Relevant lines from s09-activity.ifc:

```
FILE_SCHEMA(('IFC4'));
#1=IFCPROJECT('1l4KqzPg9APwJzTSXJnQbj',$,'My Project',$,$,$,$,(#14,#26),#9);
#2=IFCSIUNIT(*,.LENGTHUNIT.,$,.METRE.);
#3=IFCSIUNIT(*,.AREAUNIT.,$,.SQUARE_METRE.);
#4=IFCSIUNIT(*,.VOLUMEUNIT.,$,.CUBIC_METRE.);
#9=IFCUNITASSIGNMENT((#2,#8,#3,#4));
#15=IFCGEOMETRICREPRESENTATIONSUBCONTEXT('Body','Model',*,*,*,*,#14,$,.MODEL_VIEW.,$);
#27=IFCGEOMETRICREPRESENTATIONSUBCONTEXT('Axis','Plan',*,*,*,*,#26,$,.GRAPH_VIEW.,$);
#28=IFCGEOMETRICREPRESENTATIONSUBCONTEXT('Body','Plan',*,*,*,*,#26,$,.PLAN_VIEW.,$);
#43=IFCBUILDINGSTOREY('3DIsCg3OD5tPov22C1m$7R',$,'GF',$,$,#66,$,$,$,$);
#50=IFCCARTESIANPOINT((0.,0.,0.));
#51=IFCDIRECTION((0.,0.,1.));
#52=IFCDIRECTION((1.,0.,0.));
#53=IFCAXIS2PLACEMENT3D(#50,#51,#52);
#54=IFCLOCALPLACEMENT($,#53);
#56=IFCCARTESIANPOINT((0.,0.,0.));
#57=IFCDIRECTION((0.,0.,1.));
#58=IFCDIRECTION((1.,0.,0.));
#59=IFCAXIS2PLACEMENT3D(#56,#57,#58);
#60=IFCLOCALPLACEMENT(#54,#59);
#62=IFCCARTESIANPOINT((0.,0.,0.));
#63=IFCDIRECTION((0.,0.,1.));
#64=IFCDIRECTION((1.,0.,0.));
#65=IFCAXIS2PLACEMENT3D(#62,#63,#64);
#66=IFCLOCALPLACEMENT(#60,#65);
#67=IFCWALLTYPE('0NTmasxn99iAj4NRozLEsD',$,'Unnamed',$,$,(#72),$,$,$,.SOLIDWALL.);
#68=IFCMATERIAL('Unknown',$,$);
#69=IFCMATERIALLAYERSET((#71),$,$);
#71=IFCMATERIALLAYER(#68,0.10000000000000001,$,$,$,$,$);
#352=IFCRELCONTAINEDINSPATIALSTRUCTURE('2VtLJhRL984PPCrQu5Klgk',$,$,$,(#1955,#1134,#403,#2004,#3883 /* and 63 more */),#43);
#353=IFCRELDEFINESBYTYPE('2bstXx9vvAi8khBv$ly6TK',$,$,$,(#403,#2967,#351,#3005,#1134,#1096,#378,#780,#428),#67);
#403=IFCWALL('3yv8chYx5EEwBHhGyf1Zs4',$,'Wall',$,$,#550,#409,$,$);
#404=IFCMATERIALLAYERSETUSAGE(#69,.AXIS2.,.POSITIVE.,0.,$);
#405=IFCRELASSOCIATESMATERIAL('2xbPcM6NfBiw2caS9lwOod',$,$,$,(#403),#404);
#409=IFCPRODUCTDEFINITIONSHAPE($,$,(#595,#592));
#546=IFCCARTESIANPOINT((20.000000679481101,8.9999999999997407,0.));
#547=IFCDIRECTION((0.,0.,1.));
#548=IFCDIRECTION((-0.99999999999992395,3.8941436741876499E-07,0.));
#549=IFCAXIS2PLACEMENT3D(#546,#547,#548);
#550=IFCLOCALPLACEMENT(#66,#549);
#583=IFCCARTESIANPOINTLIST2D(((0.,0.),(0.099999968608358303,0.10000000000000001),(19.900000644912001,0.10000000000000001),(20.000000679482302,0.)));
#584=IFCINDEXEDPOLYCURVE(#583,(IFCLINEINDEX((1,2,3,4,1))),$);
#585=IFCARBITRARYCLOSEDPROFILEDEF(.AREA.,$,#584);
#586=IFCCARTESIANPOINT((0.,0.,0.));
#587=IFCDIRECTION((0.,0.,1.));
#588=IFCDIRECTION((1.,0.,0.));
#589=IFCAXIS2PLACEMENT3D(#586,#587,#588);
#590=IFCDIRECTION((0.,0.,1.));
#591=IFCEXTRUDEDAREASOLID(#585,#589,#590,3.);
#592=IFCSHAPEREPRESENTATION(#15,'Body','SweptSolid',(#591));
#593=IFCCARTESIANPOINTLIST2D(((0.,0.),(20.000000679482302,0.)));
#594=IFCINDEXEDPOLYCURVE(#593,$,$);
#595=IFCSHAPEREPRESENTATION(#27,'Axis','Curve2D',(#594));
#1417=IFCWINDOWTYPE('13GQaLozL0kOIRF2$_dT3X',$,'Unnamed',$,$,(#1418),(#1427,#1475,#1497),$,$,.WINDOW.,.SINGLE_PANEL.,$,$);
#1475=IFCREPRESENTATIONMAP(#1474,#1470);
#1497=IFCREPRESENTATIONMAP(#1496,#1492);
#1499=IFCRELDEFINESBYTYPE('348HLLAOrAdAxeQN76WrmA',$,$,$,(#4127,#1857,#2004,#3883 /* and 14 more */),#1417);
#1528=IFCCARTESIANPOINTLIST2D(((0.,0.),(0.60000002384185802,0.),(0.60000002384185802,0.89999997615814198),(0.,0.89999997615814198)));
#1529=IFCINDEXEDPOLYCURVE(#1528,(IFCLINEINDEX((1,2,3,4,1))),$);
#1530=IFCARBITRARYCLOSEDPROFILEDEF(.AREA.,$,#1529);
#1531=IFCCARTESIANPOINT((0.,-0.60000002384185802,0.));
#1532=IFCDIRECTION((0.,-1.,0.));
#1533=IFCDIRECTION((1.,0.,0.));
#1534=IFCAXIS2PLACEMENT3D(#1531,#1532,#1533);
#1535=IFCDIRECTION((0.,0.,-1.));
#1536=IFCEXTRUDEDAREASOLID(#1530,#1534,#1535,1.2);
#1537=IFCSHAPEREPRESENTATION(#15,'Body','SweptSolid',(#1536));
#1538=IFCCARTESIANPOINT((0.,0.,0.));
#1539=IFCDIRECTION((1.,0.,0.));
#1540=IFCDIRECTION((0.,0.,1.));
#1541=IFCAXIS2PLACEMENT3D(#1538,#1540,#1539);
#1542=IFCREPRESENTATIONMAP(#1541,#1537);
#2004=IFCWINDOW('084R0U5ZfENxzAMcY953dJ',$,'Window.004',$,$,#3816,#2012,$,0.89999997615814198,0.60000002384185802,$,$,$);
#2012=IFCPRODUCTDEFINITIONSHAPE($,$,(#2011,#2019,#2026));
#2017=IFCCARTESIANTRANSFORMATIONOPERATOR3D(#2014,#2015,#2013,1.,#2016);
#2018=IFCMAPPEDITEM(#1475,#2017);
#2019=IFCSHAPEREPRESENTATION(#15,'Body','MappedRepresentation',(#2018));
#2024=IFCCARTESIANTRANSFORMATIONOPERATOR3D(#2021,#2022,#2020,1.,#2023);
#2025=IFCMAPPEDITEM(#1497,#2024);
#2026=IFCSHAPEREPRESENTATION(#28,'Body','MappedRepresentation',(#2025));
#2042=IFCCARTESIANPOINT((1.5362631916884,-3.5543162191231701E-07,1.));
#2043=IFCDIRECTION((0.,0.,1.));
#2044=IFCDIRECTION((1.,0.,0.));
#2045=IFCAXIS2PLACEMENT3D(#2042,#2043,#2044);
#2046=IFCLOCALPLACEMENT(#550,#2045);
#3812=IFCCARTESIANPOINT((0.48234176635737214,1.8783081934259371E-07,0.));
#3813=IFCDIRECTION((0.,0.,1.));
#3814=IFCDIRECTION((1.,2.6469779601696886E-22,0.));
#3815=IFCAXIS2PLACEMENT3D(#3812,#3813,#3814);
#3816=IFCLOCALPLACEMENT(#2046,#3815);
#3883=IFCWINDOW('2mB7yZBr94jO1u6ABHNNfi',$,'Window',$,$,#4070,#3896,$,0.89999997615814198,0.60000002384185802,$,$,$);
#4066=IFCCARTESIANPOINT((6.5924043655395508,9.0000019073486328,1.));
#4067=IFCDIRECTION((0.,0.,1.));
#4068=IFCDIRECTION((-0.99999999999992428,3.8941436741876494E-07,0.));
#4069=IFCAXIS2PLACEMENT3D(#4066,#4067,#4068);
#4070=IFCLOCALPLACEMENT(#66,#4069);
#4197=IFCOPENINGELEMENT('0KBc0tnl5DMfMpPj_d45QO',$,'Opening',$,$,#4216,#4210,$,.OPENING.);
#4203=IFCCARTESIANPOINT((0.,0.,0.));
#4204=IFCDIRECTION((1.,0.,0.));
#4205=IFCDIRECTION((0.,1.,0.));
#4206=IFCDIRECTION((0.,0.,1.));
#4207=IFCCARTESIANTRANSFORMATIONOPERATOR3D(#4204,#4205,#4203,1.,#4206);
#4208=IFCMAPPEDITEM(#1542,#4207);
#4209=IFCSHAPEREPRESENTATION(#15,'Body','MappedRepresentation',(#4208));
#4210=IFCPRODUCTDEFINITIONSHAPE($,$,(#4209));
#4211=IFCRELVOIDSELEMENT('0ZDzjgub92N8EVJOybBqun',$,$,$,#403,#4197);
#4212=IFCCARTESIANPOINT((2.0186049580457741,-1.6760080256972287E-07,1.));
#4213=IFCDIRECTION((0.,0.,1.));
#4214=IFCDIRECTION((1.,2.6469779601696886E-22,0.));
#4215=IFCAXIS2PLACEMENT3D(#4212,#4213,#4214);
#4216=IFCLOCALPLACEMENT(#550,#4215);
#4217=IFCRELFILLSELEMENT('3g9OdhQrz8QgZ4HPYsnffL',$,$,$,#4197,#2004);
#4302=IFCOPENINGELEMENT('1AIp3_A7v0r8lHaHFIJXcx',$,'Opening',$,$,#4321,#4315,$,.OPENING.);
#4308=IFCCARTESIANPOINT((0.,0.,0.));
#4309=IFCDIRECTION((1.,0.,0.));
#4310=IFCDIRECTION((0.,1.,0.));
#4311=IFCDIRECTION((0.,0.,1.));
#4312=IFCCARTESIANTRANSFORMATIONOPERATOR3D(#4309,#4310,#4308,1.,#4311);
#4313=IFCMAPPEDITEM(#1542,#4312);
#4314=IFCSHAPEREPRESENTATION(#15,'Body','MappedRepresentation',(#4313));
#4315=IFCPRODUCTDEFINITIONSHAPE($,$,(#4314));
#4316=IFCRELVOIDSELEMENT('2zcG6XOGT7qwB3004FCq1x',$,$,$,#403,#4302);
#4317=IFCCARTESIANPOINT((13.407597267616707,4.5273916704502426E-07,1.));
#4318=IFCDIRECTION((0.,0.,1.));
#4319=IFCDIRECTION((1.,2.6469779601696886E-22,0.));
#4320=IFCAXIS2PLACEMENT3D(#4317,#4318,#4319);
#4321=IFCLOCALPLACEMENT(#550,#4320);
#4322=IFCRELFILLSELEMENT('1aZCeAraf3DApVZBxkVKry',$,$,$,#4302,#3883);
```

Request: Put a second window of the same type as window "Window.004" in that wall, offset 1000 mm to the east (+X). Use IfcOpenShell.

```python
import ifcopenshell
import ifcopenshell.api.feature
import ifcopenshell.api.geometry
import ifcopenshell.api.root
import ifcopenshell.geom
import ifcopenshell.util.element
import ifcopenshell.util.placement
import ifcopenshell.util.shape
import ifcopenshell.util.unit

model = ifcopenshell.open("s09-activity.ifc")
unit_scale = ifcopenshell.util.unit.calculate_unit_scale(model)
settings = ifcopenshell.geom.settings()


def volume(element):
    """Net volume in cubic metres, openings subtracted."""
    shape = ifcopenshell.geom.create_shape(settings, element)
    return ifcopenshell.util.shape.get_volume(shape.geometry)


window = model.by_guid("084R0U5ZfENxzAMcY953dJ")
opening = window.FillsVoids[0].RelatingOpeningElement
wall = opening.VoidsElements[0].RelatingBuildingElement
before = volume(wall)
shift = ifcopenshell.util.placement.get_local_placement(wall.ObjectPlacement)[:3, 0] * -1 / unit_scale

# copy_class copies the void relationship, type, container and properties, but no geometry.
new_opening = ifcopenshell.api.root.copy_class(model, product=opening)
new_opening.Representation = ifcopenshell.util.element.copy_deep(
    model, opening.Representation, exclude=["IfcGeometricRepresentationContext", "IfcRepresentationMap"]
)
new_window = ifcopenshell.api.root.copy_class(model, product=window)
new_window.Representation = ifcopenshell.util.element.copy_deep(
    model, window.Representation, exclude=["IfcGeometricRepresentationContext", "IfcRepresentationMap"]
)
ifcopenshell.api.feature.add_filling(model, opening=new_opening, element=new_window)

for old, new in ((opening, new_opening), (window, new_window)):
    matrix = ifcopenshell.util.placement.get_local_placement(old.ObjectPlacement)
    matrix[:3, 3] += shift
    ifcopenshell.api.geometry.edit_object_placement(model, product=new, matrix=matrix, is_si=False)

after = volume(wall)

print(f"wall volume {before:.3f} -> {after:.3f} m3")

model.write("s09-activity-out.ifc")
```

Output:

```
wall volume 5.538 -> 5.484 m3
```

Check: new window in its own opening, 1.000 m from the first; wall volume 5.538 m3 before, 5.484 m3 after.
